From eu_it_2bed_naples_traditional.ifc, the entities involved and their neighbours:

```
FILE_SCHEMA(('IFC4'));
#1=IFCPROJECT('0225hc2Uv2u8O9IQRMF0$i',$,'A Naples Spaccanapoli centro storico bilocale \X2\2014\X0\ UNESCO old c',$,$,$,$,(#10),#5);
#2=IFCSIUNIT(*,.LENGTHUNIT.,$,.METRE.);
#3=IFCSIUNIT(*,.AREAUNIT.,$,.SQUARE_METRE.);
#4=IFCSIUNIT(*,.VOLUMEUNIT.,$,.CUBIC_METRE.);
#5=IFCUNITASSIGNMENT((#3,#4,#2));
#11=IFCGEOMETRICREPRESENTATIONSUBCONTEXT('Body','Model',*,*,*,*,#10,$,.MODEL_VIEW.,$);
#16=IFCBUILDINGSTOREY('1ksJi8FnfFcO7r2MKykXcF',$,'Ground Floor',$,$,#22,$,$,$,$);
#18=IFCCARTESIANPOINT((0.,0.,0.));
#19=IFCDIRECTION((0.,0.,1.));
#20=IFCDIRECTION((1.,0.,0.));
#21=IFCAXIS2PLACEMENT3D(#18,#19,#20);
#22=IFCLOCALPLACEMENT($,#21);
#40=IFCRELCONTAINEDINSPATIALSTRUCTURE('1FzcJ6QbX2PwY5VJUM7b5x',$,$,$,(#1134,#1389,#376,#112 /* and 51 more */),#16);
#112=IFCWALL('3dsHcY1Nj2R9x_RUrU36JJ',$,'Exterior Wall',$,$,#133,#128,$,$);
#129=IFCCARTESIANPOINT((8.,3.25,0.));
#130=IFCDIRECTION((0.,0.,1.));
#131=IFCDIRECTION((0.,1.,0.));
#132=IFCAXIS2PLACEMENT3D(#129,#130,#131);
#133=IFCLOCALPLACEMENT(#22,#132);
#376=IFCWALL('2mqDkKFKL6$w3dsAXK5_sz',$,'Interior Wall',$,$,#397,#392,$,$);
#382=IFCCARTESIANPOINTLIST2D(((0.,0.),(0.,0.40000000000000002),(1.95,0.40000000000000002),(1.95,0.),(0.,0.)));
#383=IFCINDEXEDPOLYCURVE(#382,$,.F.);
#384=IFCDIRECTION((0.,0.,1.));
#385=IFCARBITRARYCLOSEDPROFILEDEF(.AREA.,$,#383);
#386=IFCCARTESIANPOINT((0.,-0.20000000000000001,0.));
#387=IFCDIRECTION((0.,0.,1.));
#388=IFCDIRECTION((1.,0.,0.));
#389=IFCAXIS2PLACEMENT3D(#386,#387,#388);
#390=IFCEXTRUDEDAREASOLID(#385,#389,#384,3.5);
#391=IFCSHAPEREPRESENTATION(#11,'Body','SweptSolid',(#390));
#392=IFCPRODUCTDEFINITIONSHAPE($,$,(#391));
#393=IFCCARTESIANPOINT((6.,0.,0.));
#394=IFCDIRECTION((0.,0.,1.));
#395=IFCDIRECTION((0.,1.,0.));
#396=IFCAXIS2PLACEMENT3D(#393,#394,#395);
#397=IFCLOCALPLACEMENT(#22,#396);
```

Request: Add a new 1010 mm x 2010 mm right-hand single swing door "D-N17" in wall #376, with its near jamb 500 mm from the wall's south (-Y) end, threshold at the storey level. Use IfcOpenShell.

```python
import numpy as np
import ifcopenshell
import ifcopenshell.api.feature
import ifcopenshell.api.geometry
import ifcopenshell.api.root
import ifcopenshell.api.spatial
import ifcopenshell.geom
import ifcopenshell.util.element
import ifcopenshell.util.placement
import ifcopenshell.util.representation
import ifcopenshell.util.shape
import ifcopenshell.util.unit

model = ifcopenshell.open("eu_it_2bed_naples_traditional.ifc")
unit_scale = ifcopenshell.util.unit.calculate_unit_scale(model)
settings = ifcopenshell.geom.settings()


def volume(element):
    """Net volume in cubic metres, openings subtracted."""
    shape = ifcopenshell.geom.create_shape(settings, element)
    return ifcopenshell.util.shape.get_volume(shape.geometry)


wall = model.by_id(376)
storey = ifcopenshell.util.element.get_container(wall, ifc_class="IfcBuildingStorey")
context = ifcopenshell.util.representation.get_context(model, "Model", "Body", "MODEL_VIEW")
before = volume(wall)

width, height, from_end, sill = 1.01, 2.01, 0.5, 0.0  # metres

# The wall runs along its own X axis, and the end named is its -X end.
wall_shape = ifcopenshell.geom.create_shape(settings, wall)
x, y, z = ifcopenshell.util.shape.get_vertices(wall_shape.geometry).T
start = x.min() + from_end
face, thickness = float(y.min()), float(y.max() - y.min())
wall_matrix = ifcopenshell.util.placement.get_local_placement(wall.ObjectPlacement)
level = ifcopenshell.util.placement.get_local_placement(storey.ObjectPlacement)[2, 3]


def in_wall(x, y):
    """Placement at x, y metres in the wall's axes, at sill height."""
    matrix = wall_matrix.copy()
    matrix[:, 3] = wall_matrix @ np.array([x / unit_scale, y / unit_scale, 0.0, 1.0])
    matrix[2, 3] = level + sill / unit_scale
    return matrix


# Opening: a box that overshoots both wall faces by 50 mm.
opening = ifcopenshell.api.root.create_entity(model, ifc_class="IfcOpeningElement", predefined_type="OPENING")
box = ifcopenshell.api.geometry.add_wall_representation(
    model, context=context, length=width, height=height, thickness=thickness + 0.1
)
ifcopenshell.api.geometry.assign_representation(model, product=opening, representation=box)
ifcopenshell.api.geometry.edit_object_placement(model, product=opening, matrix=in_wall(start, face - 0.05), is_si=False)
ifcopenshell.api.feature.add_feature(model, feature=opening, element=wall)

door = ifcopenshell.api.root.create_entity(model, ifc_class="IfcDoor", name="D-N17", predefined_type="DOOR")
door.OverallWidth, door.OverallHeight = width / unit_scale, height / unit_scale
door.OperationType = "SINGLE_SWING_RIGHT"
body = ifcopenshell.api.geometry.add_door_representation(
    model,
    context=context,
    overall_width=door.OverallWidth,
    overall_height=door.OverallHeight,
    operation_type="SINGLE_SWING_RIGHT",
    lining_properties={"LiningDepth": thickness / unit_scale, "ThresholdDepth": thickness / unit_scale},
)
ifcopenshell.api.geometry.assign_representation(model, product=door, representation=body)
ifcopenshell.api.spatial.assign_container(model, products=[door], relating_structure=storey)
ifcopenshell.api.feature.add_filling(model, opening=opening, element=door)

# The lining spans the wall, so the door starts at the wall face.
ifcopenshell.api.geometry.edit_object_placement(model, product=door, matrix=in_wall(start, face), is_si=False)

after = volume(wall)

print(f"wall volume {before:.3f} -> {after:.3f} m3")

model.write("eu_it_2bed_naples_traditional_v2.ifc")
```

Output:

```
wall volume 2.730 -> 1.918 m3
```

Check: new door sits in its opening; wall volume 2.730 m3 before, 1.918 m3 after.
